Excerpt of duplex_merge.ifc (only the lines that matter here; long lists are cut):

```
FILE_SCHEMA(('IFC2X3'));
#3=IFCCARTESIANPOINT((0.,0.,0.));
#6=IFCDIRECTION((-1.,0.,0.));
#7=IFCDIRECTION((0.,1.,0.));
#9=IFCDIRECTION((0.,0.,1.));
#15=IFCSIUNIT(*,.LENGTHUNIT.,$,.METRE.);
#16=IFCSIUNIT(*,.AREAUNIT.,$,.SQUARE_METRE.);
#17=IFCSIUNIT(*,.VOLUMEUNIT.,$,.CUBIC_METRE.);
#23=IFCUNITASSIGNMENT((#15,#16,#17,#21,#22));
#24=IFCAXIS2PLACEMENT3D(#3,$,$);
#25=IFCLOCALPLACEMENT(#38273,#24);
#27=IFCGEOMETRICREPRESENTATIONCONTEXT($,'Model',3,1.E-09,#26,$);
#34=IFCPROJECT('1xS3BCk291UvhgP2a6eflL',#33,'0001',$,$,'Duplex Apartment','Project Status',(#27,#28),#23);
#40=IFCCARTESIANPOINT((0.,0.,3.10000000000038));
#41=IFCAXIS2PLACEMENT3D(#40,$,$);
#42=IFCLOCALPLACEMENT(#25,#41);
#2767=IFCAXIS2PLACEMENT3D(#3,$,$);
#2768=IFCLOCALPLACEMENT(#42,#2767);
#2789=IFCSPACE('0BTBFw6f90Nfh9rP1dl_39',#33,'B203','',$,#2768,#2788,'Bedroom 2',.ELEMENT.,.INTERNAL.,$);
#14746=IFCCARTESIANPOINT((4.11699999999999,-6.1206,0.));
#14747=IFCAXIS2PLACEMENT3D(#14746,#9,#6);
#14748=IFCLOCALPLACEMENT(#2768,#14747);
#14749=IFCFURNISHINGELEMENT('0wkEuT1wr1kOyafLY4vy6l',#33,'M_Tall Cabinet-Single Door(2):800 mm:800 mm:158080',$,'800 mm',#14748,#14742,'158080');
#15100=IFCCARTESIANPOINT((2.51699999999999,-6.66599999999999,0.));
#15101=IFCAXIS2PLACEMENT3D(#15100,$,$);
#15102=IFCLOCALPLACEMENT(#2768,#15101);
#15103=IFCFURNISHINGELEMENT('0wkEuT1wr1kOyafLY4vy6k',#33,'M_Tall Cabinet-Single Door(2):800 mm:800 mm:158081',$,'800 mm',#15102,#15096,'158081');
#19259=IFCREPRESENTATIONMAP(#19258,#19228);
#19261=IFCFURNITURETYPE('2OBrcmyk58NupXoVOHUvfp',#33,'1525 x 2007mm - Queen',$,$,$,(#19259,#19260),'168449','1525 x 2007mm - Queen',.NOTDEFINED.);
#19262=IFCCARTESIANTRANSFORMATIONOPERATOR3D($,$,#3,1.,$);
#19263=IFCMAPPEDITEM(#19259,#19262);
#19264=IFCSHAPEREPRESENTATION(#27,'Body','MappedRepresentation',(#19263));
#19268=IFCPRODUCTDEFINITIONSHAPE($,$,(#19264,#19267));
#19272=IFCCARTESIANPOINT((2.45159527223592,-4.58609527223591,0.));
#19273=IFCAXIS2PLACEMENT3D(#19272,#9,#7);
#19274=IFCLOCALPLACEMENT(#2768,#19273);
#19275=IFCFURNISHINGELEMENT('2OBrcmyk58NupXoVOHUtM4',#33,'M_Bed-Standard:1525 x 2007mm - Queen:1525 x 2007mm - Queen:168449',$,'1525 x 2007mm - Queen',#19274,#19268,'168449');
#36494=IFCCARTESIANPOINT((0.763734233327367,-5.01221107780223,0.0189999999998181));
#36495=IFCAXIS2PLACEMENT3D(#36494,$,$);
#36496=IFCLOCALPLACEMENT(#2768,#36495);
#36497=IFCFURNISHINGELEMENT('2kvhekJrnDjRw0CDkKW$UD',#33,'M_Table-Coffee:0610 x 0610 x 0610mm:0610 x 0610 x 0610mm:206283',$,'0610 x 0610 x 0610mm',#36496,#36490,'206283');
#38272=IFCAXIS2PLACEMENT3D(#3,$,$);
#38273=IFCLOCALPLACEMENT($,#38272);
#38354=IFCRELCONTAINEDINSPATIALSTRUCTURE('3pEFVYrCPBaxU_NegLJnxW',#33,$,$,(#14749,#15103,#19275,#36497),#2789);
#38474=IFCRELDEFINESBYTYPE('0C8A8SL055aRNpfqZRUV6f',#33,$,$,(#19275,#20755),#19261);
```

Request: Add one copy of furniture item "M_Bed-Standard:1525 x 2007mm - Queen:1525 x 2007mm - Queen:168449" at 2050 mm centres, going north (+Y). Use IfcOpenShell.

```python
import numpy as np
import ifcopenshell
import ifcopenshell.api.geometry
import ifcopenshell.api.root
import ifcopenshell.util.element
import ifcopenshell.util.placement
import ifcopenshell.util.unit

model = ifcopenshell.open("duplex_merge.ifc")
unit_scale = ifcopenshell.util.unit.calculate_unit_scale(model)


def reuse_history(source, copy):
    """copy_class also copies each property set's owner history, people and application; keep the originals."""
    for rel in copy.IsDefinedBy:
        if rel.is_a("IfcRelDefinesByProperties") and (history := rel.RelatingPropertyDefinition.OwnerHistory):
            rel.RelatingPropertyDefinition.OwnerHistory = source.OwnerHistory
            ifcopenshell.util.element.remove_deep2(model, history)


source = model.by_guid("2OBrcmyk58NupXoVOHUtM4")
base = ifcopenshell.util.placement.get_local_placement(source.ObjectPlacement)
step = np.array([0.0, 1.0, 0.0]) * 2.05 / unit_scale

for i in range(1, 2):
    copy = ifcopenshell.api.root.copy_class(model, product=source)
    copy.Representation = ifcopenshell.util.element.copy_deep(
        model, source.Representation, exclude=["IfcGeometricRepresentationContext", "IfcRepresentationMap"]
    )
    copy.Name = "M_Bed-Standard:1525 x 2007mm - Queen:1525 x 2007mm - Queen"
    copy.Tag = None
    reuse_history(source, copy)
    matrix = base.copy()
    matrix[:3, 3] += i * step
    print("added at", matrix[:3, 3].round(3) + 0.0)
    ifcopenshell.api.geometry.edit_object_placement(model, product=copy, matrix=matrix, is_si=False)

model.write("duplex_merge_v2.ifc")
```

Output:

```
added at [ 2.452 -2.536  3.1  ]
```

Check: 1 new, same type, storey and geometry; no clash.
